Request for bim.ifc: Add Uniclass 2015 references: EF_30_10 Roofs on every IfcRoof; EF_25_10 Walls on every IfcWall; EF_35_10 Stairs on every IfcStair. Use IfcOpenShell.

First a look at what the model holds.

```python
import ifcopenshell

model = ifcopenshell.open("bim.ifc")
print(model.schema)
print("classifications:", [c.Name for c in model.by_type("IfcClassification")])
for ifc_class in ("IfcDoor", "IfcRoof", "IfcStair", "IfcWall", "IfcWindow"):
    print(ifc_class, len(model.by_type(ifc_class)))
```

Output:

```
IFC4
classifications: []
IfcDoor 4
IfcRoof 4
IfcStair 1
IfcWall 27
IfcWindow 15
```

```python
import ifcopenshell
import ifcopenshell.api.classification

model = ifcopenshell.open("bim.ifc")

system = ifcopenshell.api.classification.add_classification(model, classification="Uniclass 2015")

codes = {
    "IfcRoof": ("EF_30_10", "Roofs"),
    "IfcWall": ("EF_25_10", "Walls"),
    "IfcStair": ("EF_35_10", "Stairs"),
}
for ifc_class, (code, name) in codes.items():
    products = model.by_type(ifc_class)
    ifcopenshell.api.classification.add_reference(
        model, products=products, classification=system, identification=code, name=name
    )
    print(code, len(products))

model.write("bim_updated.ifc")
```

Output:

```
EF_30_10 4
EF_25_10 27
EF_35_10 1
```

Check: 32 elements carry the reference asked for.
